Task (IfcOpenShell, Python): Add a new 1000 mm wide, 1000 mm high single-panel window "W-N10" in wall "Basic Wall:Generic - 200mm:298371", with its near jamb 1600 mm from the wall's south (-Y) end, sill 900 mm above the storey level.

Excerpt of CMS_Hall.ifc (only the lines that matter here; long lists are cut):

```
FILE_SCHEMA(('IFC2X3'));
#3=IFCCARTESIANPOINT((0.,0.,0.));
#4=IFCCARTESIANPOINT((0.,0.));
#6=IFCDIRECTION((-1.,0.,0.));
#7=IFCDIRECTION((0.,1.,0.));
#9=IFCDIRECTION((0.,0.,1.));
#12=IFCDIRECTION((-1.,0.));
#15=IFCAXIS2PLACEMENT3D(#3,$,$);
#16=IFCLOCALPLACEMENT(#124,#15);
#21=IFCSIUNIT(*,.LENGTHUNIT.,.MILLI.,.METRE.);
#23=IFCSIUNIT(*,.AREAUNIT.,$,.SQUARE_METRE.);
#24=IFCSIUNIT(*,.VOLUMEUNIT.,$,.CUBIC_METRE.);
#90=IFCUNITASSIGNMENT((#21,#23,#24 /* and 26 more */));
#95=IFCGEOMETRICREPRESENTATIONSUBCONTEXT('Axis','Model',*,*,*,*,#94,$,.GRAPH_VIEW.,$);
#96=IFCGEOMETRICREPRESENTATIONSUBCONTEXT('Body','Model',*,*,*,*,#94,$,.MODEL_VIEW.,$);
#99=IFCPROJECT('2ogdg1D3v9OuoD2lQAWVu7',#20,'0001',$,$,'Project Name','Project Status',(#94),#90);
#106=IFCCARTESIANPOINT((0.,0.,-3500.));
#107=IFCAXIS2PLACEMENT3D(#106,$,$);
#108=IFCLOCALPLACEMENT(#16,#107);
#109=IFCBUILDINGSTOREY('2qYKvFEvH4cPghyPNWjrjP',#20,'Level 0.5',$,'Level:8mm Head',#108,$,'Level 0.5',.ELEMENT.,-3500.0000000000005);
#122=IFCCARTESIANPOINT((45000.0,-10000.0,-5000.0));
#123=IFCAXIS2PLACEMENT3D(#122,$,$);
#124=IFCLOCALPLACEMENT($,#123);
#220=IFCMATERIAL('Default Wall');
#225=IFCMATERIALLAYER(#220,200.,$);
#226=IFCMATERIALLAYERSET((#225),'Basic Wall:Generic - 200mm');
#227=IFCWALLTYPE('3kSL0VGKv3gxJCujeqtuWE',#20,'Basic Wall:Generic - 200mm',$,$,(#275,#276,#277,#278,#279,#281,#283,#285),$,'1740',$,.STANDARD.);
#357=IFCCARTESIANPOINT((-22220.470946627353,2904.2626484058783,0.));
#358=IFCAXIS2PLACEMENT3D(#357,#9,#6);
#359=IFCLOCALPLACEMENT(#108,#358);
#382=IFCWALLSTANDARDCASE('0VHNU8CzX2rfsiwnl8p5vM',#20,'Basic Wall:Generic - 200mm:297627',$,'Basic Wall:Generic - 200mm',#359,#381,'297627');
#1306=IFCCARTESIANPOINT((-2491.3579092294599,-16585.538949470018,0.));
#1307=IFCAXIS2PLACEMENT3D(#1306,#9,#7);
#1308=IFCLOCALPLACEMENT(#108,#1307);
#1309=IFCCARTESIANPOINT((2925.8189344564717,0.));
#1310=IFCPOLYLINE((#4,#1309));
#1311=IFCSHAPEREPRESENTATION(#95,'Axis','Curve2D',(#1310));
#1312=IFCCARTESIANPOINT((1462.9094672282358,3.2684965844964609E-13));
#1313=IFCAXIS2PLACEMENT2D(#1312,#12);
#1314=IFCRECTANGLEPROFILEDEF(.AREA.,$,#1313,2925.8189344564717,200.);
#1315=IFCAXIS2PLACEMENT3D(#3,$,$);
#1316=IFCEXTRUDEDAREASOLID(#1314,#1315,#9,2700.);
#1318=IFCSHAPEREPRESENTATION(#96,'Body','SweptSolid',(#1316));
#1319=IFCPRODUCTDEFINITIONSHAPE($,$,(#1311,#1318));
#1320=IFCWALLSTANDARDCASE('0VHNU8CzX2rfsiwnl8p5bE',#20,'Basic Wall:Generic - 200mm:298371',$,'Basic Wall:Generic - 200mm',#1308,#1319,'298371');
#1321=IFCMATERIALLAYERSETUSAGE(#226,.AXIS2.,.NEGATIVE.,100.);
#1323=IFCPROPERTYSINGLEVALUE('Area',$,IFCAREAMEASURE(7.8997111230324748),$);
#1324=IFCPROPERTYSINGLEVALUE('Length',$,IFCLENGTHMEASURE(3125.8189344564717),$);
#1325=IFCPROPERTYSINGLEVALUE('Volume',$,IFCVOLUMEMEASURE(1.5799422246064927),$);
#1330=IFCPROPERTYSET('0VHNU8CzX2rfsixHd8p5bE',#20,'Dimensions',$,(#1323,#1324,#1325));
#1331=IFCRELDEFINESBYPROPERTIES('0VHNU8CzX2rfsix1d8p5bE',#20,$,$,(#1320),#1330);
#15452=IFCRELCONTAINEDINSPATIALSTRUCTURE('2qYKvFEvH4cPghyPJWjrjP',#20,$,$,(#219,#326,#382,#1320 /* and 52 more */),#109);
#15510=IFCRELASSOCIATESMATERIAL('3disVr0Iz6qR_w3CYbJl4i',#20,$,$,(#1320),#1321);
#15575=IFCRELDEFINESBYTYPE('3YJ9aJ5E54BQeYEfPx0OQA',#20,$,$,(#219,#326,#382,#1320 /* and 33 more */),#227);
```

```python
import numpy as np
import ifcopenshell
import ifcopenshell.api.feature
import ifcopenshell.api.geometry
import ifcopenshell.api.pset
import ifcopenshell.api.root
import ifcopenshell.api.spatial
import ifcopenshell.api.type
import ifcopenshell.geom
import ifcopenshell.util.element
import ifcopenshell.util.placement
import ifcopenshell.util.representation
import ifcopenshell.util.shape
import ifcopenshell.util.unit

model = ifcopenshell.open("CMS_Hall.ifc")
unit_scale = ifcopenshell.util.unit.calculate_unit_scale(model)
area_scale = ifcopenshell.util.unit.calculate_unit_scale(model, "AREAUNIT")
volume_scale = ifcopenshell.util.unit.calculate_unit_scale(model, "VOLUMEUNIT")
settings = ifcopenshell.geom.settings()


def volume(element):
    """Net volume in cubic metres, openings subtracted."""
    shape = ifcopenshell.geom.create_shape(settings, element)
    return ifcopenshell.util.shape.get_volume(shape.geometry)


wall = model.by_guid("0VHNU8CzX2rfsiwnl8p5bE")
storey = ifcopenshell.util.element.get_container(wall, ifc_class="IfcBuildingStorey")
context = ifcopenshell.util.representation.get_context(model, "Model", "Body", "MODEL_VIEW")
before = volume(wall)

width, height, from_end, sill = 1, 1, 1.6, 0.9  # metres

# The wall runs along its own X axis, and the end named is its -X end.
wall_shape = ifcopenshell.geom.create_shape(settings, wall)
x, y, z = ifcopenshell.util.shape.get_vertices(wall_shape.geometry).T
start = x.min() + from_end
face, thickness = float(y.min()), float(y.max() - y.min())
wall_matrix = ifcopenshell.util.placement.get_local_placement(wall.ObjectPlacement)
level = ifcopenshell.util.placement.get_local_placement(storey.ObjectPlacement)[2, 3]


def in_wall(x, y):
    """Placement at x, y metres in the wall's axes, at sill height."""
    matrix = wall_matrix.copy()
    matrix[:, 3] = wall_matrix @ np.array([x / unit_scale, y / unit_scale, 0.0, 1.0])
    matrix[2, 3] = level + sill / unit_scale
    return matrix


# Opening: a box that overshoots both wall faces by 50 mm.
opening = ifcopenshell.api.root.create_entity(model, ifc_class="IfcOpeningElement")
box = ifcopenshell.api.geometry.add_wall_representation(
    model, context=context, length=width, height=height, thickness=thickness + 0.1
)
ifcopenshell.api.geometry.assign_representation(model, product=opening, representation=box)
ifcopenshell.api.geometry.edit_object_placement(model, product=opening, matrix=in_wall(start, face - 0.05), is_si=False)
ifcopenshell.api.feature.add_feature(model, feature=opening, element=wall)

window = ifcopenshell.api.root.create_entity(model, ifc_class="IfcWindow", name="W-N10")
window.OverallWidth, window.OverallHeight = width / unit_scale, height / unit_scale
body = ifcopenshell.api.geometry.add_window_representation(
    model,
    context=context,
    overall_width=window.OverallWidth,
    overall_height=window.OverallHeight,
    partition_type="SINGLE_PANEL",
)
ifcopenshell.api.geometry.assign_representation(model, product=window, representation=body)
ifcopenshell.api.spatial.assign_container(model, products=[window], relating_structure=storey)
fills = ifcopenshell.api.feature.add_filling(model, opening=opening, element=window)
fills.OwnerHistory = window.OwnerHistory  # required in IFC2X3

# IFC2X3 keeps the operation on the window style.
style = ifcopenshell.api.root.create_entity(model, ifc_class="IfcWindowStyle", name="W-N10")
style.OperationType, style.ConstructionType = "SINGLE_PANEL", "NOTDEFINED"
style.ParameterTakesPrecedence = style.Sizeable = False
ifcopenshell.api.type.assign_type(model, related_objects=[window], relating_type=style)

# Centre the window in the wall's thickness.
ifcopenshell.api.geometry.edit_object_placement(model, product=window, matrix=in_wall(start, face), is_si=False)
window_shape = ifcopenshell.geom.create_shape(settings, window)
depth = ifcopenshell.util.shape.get_vertices(window_shape.geometry)[:, 1]
offset = face + thickness / 2 - (depth.min() + depth.max()) / 2
ifcopenshell.api.geometry.edit_object_placement(model, product=window, matrix=in_wall(start, offset), is_si=False)

after = volume(wall)

# Update the wall's stored quantities.
pset = model.by_id(ifcopenshell.util.element.get_pset(wall, "Dimensions", should_inherit=False)["id"])
ifcopenshell.api.pset.edit_pset(model, pset=pset, properties={
    "Area": model.create_entity("IfcAreaMeasure", after / thickness / area_scale),
    "Volume": model.create_entity("IfcVolumeMeasure", after / volume_scale),
})

print(f"wall volume {before:.3f} -> {after:.3f} m3")

model.write("CMS_Hall_edited.ifc")
```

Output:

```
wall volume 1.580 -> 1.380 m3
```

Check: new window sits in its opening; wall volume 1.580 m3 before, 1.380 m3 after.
